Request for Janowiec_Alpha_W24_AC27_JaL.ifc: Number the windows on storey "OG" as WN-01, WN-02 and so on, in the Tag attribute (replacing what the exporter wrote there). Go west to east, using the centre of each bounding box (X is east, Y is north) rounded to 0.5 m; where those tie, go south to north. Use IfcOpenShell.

First a look at what the model holds.

```python
import ifcopenshell
import ifcopenshell.util.element
import ifcopenshell.util.placement

model = ifcopenshell.open("Janowiec_Alpha_W24_AC27_JaL.ifc")
print(model.schema)
storey = next(s for s in model.by_type("IfcBuildingStorey") if s.Name == "OG")
windows = [e for e in ifcopenshell.util.element.get_decomposition(storey) if e.is_a("IfcWindow")]
for e in sorted(windows, key=lambda e: e.id()):
    origin = ifcopenshell.util.placement.get_local_placement(e.ObjectPlacement)[:3, 3]
    print(e.id(), e.Tag, e.Name, origin.round(2) + 0.0, sep=" | ")
```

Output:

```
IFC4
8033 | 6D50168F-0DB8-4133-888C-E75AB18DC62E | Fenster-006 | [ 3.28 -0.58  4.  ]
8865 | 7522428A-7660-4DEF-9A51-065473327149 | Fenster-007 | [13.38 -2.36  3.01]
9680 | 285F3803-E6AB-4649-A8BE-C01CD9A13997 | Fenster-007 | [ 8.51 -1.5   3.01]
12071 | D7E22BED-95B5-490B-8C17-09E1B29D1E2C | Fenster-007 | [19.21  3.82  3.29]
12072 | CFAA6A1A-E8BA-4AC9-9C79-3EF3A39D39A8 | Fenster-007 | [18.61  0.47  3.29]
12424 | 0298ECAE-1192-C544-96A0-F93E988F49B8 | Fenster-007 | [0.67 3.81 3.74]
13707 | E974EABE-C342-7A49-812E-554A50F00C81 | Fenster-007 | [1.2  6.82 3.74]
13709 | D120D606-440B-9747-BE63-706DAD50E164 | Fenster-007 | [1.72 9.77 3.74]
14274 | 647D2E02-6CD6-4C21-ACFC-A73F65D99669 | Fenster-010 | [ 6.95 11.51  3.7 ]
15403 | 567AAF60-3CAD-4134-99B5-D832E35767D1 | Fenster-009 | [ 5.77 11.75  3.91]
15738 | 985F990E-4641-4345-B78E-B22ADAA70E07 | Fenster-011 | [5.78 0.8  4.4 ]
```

```python
import ifcopenshell
import ifcopenshell.geom
import ifcopenshell.util.element
import ifcopenshell.util.shape

model = ifcopenshell.open("Janowiec_Alpha_W24_AC27_JaL.ifc")
settings = ifcopenshell.geom.settings()
settings.set("use-world-coords", True)


def centre(element):
    shape = ifcopenshell.geom.create_shape(settings, element)
    return ifcopenshell.util.shape.get_bbox_centroid(shape.geometry)


storey = next(s for s in model.by_type("IfcBuildingStorey") if s.Name == "OG")
windows = [e for e in ifcopenshell.util.element.get_decomposition(storey) if e.is_a("IfcWindow")]

# Insertion points can sit at a corner or the storey origin, so sort by the geometry (in metres).
centres = {e: centre(e) for e in windows}
windows.sort(key=lambda e: (round(centres[e][0] / 0.5), centres[e][1]))

for i, e in enumerate(windows, start=1):
    number = f"WN-{i:02d}"
    e.Tag = number
    print(e.id(), number)

model.write("Janowiec_Alpha_W24_AC27_JaL_v2.ifc")
```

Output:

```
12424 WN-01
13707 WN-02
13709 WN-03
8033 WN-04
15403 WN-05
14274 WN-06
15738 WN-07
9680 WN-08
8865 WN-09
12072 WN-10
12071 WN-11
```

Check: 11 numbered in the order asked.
